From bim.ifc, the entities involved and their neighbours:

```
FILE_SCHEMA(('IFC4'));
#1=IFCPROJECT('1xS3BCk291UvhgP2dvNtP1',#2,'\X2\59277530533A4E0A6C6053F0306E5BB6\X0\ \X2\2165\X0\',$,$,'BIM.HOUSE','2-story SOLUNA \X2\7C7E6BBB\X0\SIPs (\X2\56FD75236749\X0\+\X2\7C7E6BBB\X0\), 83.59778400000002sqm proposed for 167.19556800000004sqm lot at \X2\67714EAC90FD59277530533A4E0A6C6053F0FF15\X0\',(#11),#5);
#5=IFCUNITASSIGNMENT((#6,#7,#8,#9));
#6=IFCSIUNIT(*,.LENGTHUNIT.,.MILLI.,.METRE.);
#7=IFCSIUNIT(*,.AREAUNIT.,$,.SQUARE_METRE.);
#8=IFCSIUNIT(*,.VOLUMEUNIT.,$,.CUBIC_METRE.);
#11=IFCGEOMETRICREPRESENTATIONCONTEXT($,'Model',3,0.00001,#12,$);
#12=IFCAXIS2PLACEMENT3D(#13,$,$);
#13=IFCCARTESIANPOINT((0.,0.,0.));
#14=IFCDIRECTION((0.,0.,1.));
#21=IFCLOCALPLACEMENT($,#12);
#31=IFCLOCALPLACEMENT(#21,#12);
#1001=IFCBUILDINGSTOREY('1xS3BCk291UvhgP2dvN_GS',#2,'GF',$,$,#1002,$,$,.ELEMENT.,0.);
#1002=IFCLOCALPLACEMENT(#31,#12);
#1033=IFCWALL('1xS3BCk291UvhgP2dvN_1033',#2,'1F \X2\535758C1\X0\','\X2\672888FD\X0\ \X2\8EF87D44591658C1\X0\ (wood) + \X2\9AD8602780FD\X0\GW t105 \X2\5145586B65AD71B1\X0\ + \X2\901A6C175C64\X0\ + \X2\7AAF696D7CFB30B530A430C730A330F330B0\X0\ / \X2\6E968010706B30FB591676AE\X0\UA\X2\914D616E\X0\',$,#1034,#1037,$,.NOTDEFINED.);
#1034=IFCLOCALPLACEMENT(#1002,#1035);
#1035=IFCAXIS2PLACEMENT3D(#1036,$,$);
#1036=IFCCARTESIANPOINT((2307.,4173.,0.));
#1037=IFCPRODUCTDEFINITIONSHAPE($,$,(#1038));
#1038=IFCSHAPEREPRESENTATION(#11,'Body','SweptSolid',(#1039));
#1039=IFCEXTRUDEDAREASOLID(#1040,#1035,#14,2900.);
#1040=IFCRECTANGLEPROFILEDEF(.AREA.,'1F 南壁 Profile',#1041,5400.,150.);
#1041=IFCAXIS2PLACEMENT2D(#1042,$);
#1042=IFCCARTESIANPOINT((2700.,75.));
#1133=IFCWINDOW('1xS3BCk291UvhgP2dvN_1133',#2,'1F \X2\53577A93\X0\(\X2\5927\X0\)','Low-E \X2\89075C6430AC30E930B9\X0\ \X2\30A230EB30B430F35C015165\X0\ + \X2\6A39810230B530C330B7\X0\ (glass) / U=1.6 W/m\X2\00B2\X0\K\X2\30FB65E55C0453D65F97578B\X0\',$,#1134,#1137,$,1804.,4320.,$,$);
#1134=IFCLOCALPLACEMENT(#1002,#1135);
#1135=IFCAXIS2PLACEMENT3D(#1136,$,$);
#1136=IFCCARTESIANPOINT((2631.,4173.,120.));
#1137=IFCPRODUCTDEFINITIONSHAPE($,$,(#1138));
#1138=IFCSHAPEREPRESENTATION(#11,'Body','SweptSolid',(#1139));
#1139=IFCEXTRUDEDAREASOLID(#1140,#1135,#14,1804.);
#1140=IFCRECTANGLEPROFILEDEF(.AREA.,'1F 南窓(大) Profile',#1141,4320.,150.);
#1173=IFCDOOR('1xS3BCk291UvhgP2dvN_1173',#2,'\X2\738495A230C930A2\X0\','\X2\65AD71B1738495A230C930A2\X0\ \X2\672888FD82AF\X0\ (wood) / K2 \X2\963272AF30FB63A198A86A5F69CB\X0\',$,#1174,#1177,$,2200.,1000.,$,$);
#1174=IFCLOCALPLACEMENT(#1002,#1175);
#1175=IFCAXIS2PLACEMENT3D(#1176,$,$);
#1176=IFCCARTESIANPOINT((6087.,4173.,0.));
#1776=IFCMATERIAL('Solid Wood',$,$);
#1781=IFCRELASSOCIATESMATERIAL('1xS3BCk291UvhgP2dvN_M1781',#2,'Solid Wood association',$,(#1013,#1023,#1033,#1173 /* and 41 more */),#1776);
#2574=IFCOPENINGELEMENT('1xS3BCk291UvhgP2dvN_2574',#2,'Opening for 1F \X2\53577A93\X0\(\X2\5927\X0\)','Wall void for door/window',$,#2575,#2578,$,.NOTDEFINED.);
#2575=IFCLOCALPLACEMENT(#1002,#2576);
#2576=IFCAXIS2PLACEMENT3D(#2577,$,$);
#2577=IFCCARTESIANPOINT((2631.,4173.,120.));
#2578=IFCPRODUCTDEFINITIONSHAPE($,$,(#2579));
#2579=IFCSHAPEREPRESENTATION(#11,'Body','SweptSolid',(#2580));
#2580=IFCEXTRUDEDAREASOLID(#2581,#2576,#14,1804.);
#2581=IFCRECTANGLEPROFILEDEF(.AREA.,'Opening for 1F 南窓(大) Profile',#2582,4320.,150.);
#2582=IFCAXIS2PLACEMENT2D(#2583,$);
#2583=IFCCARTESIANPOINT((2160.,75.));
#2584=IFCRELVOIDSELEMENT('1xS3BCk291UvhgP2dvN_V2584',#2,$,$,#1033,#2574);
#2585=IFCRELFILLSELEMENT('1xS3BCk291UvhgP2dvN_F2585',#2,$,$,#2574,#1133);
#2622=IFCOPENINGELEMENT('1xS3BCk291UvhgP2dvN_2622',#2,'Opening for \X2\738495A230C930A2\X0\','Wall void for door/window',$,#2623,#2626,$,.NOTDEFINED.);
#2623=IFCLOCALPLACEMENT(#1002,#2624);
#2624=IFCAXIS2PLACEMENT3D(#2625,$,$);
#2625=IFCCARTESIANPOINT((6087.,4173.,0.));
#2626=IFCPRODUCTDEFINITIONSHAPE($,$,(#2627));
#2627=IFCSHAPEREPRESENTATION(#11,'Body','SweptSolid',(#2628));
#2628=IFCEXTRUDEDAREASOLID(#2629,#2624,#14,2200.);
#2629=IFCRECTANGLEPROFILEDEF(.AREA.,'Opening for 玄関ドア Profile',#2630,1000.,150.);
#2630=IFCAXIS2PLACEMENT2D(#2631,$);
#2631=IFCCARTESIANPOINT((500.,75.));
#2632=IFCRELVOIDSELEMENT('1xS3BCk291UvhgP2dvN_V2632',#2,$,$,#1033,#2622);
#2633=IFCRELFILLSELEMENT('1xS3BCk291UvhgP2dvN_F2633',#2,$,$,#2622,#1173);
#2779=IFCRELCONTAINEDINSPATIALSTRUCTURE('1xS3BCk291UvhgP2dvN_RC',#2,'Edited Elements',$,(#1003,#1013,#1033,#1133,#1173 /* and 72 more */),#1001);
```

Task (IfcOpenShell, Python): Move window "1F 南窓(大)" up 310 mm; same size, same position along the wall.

```python
import numpy as np
import ifcopenshell
import ifcopenshell.api.geometry
import ifcopenshell.util.placement
import ifcopenshell.util.unit

model = ifcopenshell.open("bim.ifc")
unit_scale = ifcopenshell.util.unit.calculate_unit_scale(model)

window = model.by_id(1133)
opening = window.FillsVoids[0].RelatingOpeningElement
dz = 0.31 / unit_scale

shift = np.array([0.0, 0.0, dz])
# The window is not placed relative to its opening, so move both.
for product in (opening, window):
    matrix = ifcopenshell.util.placement.get_local_placement(product.ObjectPlacement)
    matrix[:3, 3] += shift
    ifcopenshell.api.geometry.edit_object_placement(model, product=product, matrix=matrix, is_si=False)

print(f"moved by {dz * unit_scale:+.3f} m")

model.write("bim_v2.ifc")
```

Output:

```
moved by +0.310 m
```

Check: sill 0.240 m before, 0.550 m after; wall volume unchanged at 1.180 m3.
